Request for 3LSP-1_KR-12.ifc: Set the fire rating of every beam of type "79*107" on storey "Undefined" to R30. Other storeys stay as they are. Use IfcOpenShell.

First a look at what the model holds.

```python
import ifcopenshell
import ifcopenshell.util.element

model = ifcopenshell.open("3LSP-1_KR-12.ifc")
print(model.schema)
storey = next(s for s in model.by_type("IfcBuildingStorey") if s.Name == "Undefined")
beams = [e for e in ifcopenshell.util.element.get_decomposition(storey) if e.is_a("IfcBeam")]
seen = {}
for e in beams:
    element_type = ifcopenshell.util.element.get_type(e)
    key = (element_type.Name if element_type != e and element_type else None, ifcopenshell.util.element.get_pset(e, "Pset_BeamCommon", "FireRating"))
    seen[key] = seen.get(key, 0) + 1
for (name, value), count in sorted(seen.items(), key=str):
    print(count, "x", name, "|", value)
```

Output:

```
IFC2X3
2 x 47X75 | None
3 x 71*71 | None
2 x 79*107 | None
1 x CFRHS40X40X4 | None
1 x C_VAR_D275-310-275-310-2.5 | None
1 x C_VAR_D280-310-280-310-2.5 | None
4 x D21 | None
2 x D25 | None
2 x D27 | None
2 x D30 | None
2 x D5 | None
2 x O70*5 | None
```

```python
import ifcopenshell
import ifcopenshell.api.pset
import ifcopenshell.util.element

model = ifcopenshell.open("3LSP-1_KR-12.ifc")

storey = next(s for s in model.by_type("IfcBuildingStorey") if s.Name == "Undefined")
beams = [e for e in ifcopenshell.util.element.get_decomposition(storey) if e.is_a("IfcBeam")]

count = 0
for e in beams:
    element_type = ifcopenshell.util.element.get_type(e)
    if element_type in (None, e) or element_type.Name != "79*107":
        continue
    found = ifcopenshell.util.element.get_pset(e, "Pset_BeamCommon", should_inherit=False)
    if found:
        pset = model.by_id(found["id"])
        if len(ifcopenshell.util.element.get_elements_by_pset(pset)) > 1:
            pset = ifcopenshell.api.pset.unshare_pset(model, products=[e], pset=pset)[0]
    else:
        pset = ifcopenshell.api.pset.add_pset(model, product=e, name="Pset_BeamCommon")
    ifcopenshell.api.pset.edit_pset(model, pset=pset, properties={"FireRating": "R30"})
    count += 1

print(count, "beams updated")

model.write("3LSP-1_KR-12_edited.ifc")
```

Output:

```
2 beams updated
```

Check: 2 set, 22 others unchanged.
